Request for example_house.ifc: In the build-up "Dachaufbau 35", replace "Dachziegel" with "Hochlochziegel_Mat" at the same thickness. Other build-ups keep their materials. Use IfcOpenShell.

First a look at what the model holds.

```python
import ifcopenshell
import ifcopenshell.util.element

model = ifcopenshell.open("example_house.ifc")
print(model.schema)
for layer_set in model.by_type("IfcMaterialLayerSet"):
    if layer_set.LayerSetName == "Dachaufbau 35":
        for layer in layer_set.MaterialLayers:
            print(layer.id(), layer.Material and layer.Material.Name, layer.LayerThickness, sep=" | ")
        print(len(ifcopenshell.util.element.get_elements_by_material(model, layer_set)), "elements and types use it")
print(sorted(m.Name for m in model.by_type("IfcMaterial") if m.Name)[:60])
```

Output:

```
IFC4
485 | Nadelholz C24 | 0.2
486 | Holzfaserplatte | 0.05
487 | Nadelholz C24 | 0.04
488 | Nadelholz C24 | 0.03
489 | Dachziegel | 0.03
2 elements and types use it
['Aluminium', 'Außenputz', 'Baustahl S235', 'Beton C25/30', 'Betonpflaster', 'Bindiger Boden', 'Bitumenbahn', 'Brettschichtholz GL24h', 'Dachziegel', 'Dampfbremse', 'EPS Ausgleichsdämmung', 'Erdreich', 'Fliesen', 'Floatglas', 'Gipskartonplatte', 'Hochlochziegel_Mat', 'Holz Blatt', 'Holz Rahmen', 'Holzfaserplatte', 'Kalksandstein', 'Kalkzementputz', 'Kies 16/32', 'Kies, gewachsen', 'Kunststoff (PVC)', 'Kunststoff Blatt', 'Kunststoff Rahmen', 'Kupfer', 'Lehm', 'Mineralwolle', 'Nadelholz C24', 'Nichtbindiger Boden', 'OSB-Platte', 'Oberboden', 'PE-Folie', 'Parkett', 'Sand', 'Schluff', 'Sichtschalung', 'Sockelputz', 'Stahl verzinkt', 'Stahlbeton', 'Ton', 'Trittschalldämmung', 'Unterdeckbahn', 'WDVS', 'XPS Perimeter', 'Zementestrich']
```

```python
import ifcopenshell
import ifcopenshell.api.material

model = ifcopenshell.open("example_house.ifc")

layer_set = next(s for s in model.by_type("IfcMaterialLayerSet") if s.LayerSetName == "Dachaufbau 35")
layer = next(l for l in layer_set.MaterialLayers if l.Material and l.Material.Name == "Dachziegel")
material = next(m for m in model.by_type("IfcMaterial") if m.Name == "Hochlochziegel_Mat")

# Point this one layer at the other material; renaming the old one would change it everywhere.
ifcopenshell.api.material.edit_layer(model, layer=layer, attributes={"Name": material.Name}, material=material)

print([l.Material.Name if l.Material else None for l in layer_set.MaterialLayers])

model.write("example_house-out.ifc")
```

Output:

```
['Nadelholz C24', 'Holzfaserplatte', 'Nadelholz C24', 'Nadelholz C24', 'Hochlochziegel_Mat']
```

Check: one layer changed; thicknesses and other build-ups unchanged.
